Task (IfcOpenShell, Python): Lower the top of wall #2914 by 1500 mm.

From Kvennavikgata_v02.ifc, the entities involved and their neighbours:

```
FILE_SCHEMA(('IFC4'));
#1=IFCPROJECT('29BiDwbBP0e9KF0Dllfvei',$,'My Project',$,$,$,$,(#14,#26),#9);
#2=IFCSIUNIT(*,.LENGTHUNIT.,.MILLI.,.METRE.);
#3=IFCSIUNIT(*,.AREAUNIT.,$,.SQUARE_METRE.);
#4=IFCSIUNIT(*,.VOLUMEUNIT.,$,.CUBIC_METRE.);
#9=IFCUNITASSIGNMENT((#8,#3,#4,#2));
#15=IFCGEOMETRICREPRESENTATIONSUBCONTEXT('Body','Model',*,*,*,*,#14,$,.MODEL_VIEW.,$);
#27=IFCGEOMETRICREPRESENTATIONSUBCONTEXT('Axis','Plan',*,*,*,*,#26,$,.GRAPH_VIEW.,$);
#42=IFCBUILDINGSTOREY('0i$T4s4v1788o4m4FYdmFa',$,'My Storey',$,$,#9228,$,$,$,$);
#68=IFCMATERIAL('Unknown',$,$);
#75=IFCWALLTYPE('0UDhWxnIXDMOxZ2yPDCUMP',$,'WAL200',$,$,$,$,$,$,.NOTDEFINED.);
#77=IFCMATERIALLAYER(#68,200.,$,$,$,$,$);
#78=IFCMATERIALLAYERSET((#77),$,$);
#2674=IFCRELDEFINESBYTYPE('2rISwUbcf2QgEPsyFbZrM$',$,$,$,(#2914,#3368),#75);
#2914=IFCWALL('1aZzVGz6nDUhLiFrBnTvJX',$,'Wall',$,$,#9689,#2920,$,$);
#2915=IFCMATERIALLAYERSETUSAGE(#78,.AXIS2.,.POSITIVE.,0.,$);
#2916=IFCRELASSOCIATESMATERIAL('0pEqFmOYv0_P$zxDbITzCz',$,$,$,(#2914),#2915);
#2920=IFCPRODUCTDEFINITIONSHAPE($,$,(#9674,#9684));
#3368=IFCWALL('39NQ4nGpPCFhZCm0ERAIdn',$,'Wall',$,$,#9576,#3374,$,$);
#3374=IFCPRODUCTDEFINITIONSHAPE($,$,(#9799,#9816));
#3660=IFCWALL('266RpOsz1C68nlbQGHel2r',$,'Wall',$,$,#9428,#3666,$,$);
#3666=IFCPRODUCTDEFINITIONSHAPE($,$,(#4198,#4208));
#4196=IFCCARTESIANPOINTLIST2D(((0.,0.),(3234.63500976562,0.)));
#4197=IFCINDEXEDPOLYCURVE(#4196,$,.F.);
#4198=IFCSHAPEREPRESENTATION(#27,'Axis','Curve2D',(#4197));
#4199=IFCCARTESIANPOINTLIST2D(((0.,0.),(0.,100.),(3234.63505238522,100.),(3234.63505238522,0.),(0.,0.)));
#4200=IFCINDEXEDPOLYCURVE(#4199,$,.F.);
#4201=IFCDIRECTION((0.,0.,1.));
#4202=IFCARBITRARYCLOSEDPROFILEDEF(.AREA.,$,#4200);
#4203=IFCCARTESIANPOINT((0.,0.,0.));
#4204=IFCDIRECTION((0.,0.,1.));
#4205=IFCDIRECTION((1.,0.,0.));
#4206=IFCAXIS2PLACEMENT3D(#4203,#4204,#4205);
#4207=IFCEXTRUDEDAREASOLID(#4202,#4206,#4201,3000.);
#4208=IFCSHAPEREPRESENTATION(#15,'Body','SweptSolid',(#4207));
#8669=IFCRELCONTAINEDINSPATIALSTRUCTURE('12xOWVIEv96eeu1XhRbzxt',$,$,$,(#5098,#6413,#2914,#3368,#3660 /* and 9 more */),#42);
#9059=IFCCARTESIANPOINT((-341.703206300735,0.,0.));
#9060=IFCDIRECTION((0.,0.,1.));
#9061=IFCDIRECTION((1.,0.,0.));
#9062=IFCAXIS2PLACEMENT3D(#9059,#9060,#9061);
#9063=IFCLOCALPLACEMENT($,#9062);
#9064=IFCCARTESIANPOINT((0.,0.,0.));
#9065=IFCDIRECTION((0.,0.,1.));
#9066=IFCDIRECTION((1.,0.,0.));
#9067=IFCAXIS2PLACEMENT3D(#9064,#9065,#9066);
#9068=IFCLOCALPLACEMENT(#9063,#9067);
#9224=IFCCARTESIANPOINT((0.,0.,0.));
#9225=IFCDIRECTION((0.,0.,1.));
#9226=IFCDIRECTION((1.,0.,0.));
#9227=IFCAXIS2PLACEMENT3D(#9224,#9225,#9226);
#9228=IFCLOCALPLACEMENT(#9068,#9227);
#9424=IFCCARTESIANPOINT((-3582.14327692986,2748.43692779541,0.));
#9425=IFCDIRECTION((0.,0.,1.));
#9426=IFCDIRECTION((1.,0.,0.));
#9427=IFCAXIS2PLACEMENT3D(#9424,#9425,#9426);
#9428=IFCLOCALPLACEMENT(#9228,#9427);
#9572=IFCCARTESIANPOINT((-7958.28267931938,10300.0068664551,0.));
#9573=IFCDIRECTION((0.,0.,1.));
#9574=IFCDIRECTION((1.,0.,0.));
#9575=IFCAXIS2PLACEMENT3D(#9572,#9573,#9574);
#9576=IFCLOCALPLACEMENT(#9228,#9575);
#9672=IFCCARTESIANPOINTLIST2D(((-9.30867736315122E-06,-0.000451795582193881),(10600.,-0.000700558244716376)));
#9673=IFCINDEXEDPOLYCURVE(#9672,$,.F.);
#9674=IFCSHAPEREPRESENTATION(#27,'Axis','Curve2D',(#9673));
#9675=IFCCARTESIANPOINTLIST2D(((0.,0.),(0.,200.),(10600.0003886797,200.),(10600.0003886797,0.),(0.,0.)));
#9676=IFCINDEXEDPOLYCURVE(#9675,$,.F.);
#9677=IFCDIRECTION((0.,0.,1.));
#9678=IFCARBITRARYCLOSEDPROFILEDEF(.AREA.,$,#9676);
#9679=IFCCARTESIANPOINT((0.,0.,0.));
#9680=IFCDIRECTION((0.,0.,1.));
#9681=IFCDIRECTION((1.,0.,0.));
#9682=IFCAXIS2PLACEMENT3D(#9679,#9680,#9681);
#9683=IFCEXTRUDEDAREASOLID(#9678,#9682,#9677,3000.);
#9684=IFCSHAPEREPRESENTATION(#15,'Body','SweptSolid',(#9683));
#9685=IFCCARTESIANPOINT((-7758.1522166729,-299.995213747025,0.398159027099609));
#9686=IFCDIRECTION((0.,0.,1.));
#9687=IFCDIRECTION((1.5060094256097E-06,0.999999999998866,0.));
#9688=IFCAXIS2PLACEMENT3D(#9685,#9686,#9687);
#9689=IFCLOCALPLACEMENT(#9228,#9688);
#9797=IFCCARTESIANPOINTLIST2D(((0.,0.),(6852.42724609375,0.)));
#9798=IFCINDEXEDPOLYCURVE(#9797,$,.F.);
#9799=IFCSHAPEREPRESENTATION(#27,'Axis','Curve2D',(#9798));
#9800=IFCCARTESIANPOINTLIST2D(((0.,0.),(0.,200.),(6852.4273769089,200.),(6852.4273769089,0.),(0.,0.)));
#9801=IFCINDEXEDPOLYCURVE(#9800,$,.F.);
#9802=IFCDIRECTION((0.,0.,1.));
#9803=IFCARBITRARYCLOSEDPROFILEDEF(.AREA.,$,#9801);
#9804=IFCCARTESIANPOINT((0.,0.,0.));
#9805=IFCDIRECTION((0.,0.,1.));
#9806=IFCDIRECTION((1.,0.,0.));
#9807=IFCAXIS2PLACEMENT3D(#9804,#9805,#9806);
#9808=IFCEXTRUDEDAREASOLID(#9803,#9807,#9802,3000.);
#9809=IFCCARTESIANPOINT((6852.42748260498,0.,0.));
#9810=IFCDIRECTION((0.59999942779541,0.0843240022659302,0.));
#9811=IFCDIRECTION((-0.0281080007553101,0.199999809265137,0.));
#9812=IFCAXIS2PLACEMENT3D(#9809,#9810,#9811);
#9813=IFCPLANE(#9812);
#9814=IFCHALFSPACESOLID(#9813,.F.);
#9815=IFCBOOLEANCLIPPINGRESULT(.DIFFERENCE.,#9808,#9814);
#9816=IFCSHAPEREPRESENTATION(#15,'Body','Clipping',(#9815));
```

```python
import ifcopenshell
import ifcopenshell.geom
import ifcopenshell.util.representation
import ifcopenshell.util.shape
import ifcopenshell.util.unit

model = ifcopenshell.open("Kvennavikgata_v02.ifc")
unit_scale = ifcopenshell.util.unit.calculate_unit_scale(model)
settings = ifcopenshell.geom.settings()


def volume(element):
    """Net volume in cubic metres, openings subtracted."""
    shape = ifcopenshell.geom.create_shape(settings, element)
    return ifcopenshell.util.shape.get_volume(shape.geometry)


wall = model.by_guid("1aZzVGz6nDUhLiFrBnTvJX")
before = volume(wall)

body = ifcopenshell.util.representation.get_representation(wall, "Model", "Body")
solid = body.Items[0]
old_height = solid.Depth
solid.Depth -= 1.5 / unit_scale
after = volume(wall)

print(f"height {old_height:g} -> {solid.Depth:g}, volume {before:.3f} -> {after:.3f} m3")

model.write("Kvennavikgata_v02_v2.ifc")
```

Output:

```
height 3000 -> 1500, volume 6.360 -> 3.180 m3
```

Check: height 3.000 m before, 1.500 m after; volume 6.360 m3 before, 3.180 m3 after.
